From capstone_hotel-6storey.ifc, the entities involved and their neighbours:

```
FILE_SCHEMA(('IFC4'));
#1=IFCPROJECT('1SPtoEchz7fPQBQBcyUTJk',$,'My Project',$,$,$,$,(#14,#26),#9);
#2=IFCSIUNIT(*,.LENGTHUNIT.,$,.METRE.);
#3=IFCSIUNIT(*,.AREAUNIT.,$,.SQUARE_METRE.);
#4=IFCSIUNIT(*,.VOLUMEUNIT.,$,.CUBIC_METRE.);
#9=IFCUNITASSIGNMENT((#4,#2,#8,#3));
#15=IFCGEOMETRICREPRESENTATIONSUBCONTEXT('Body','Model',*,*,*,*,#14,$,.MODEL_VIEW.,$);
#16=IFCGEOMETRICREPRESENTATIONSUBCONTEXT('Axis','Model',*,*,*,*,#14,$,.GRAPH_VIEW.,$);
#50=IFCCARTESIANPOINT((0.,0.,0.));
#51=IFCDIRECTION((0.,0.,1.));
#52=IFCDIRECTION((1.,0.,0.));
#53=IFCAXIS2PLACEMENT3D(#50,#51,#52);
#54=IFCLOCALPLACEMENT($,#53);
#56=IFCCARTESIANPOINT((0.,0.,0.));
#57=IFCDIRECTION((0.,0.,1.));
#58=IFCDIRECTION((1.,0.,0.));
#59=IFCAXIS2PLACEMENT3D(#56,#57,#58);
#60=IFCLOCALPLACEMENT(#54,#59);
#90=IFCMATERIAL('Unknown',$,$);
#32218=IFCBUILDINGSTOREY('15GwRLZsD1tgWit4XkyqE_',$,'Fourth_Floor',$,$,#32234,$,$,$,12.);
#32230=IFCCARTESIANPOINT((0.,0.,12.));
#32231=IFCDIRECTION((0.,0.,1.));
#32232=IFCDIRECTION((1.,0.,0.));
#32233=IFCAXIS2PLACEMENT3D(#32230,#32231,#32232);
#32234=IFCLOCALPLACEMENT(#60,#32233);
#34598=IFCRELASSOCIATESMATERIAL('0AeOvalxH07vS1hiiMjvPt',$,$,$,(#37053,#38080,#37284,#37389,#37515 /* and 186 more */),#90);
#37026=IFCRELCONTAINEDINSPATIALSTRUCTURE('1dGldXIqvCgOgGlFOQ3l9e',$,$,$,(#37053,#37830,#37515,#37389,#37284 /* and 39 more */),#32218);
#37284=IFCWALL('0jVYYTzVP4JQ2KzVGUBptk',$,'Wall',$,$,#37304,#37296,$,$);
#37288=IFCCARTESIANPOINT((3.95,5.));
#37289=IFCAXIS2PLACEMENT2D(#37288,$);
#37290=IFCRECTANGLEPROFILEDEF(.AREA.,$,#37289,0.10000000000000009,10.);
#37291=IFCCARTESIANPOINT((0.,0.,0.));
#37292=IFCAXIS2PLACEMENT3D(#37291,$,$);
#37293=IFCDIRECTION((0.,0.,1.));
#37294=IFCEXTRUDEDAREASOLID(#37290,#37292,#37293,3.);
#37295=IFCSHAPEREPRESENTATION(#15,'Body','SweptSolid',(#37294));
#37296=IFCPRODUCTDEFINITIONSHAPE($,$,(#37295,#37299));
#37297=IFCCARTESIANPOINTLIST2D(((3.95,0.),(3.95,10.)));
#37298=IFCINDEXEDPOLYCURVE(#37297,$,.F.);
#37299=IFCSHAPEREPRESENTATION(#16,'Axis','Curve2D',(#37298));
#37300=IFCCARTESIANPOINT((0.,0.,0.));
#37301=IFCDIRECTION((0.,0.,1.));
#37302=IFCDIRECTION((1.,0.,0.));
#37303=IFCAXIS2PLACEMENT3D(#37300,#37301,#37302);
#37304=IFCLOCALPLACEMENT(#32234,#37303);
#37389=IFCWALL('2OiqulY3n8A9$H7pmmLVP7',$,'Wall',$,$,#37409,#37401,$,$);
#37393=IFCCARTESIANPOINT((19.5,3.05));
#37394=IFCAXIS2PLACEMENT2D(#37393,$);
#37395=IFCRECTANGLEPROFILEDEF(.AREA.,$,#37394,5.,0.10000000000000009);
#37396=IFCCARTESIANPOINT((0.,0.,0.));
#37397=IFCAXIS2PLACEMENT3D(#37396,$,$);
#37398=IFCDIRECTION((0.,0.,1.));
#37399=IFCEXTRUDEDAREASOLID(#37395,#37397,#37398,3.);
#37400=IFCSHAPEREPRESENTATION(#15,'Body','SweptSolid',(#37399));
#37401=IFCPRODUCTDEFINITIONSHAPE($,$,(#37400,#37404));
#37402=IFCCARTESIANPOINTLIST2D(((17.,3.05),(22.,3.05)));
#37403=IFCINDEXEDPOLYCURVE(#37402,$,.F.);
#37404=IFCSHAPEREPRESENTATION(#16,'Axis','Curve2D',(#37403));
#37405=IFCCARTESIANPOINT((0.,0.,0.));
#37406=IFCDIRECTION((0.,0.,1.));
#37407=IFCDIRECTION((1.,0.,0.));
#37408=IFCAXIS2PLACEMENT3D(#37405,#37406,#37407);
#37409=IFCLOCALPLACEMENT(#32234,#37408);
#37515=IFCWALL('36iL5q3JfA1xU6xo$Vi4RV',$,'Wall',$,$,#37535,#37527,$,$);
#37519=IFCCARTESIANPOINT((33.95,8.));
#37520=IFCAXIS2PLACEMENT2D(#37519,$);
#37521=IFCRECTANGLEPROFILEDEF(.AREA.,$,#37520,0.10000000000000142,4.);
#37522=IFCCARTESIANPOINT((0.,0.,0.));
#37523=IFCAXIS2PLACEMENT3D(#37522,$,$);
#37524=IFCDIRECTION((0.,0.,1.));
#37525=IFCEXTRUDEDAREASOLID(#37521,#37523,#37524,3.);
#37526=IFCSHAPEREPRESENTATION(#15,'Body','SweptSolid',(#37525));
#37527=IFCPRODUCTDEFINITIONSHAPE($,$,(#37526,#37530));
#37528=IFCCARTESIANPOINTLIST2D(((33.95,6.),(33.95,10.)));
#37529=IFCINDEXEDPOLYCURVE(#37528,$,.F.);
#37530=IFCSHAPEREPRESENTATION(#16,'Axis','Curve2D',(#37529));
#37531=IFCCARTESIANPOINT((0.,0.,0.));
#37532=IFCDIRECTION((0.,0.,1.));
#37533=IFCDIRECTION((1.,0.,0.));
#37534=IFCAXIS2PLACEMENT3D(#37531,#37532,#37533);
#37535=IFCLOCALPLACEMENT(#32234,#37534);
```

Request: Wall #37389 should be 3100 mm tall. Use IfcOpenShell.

```python
import ifcopenshell
import ifcopenshell.geom
import ifcopenshell.util.representation
import ifcopenshell.util.shape

model = ifcopenshell.open("capstone_hotel-6storey.ifc")
settings = ifcopenshell.geom.settings()


def volume(element):
    """Net volume in cubic metres, openings subtracted."""
    shape = ifcopenshell.geom.create_shape(settings, element)
    return ifcopenshell.util.shape.get_volume(shape.geometry)


wall = model.by_guid("2OiqulY3n8A9$H7pmmLVP7")
before = volume(wall)

body = ifcopenshell.util.representation.get_representation(wall, "Model", "Body")
solid = body.Items[0]
old_height = solid.Depth
solid.Depth = 3.1
after = volume(wall)

print(f"height {old_height:g} -> {solid.Depth:g}, volume {before:.3f} -> {after:.3f} m3")

model.write("capstone_hotel-6storey_v2.ifc")
```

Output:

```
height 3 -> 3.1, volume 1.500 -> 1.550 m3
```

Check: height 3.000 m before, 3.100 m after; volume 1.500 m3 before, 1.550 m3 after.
